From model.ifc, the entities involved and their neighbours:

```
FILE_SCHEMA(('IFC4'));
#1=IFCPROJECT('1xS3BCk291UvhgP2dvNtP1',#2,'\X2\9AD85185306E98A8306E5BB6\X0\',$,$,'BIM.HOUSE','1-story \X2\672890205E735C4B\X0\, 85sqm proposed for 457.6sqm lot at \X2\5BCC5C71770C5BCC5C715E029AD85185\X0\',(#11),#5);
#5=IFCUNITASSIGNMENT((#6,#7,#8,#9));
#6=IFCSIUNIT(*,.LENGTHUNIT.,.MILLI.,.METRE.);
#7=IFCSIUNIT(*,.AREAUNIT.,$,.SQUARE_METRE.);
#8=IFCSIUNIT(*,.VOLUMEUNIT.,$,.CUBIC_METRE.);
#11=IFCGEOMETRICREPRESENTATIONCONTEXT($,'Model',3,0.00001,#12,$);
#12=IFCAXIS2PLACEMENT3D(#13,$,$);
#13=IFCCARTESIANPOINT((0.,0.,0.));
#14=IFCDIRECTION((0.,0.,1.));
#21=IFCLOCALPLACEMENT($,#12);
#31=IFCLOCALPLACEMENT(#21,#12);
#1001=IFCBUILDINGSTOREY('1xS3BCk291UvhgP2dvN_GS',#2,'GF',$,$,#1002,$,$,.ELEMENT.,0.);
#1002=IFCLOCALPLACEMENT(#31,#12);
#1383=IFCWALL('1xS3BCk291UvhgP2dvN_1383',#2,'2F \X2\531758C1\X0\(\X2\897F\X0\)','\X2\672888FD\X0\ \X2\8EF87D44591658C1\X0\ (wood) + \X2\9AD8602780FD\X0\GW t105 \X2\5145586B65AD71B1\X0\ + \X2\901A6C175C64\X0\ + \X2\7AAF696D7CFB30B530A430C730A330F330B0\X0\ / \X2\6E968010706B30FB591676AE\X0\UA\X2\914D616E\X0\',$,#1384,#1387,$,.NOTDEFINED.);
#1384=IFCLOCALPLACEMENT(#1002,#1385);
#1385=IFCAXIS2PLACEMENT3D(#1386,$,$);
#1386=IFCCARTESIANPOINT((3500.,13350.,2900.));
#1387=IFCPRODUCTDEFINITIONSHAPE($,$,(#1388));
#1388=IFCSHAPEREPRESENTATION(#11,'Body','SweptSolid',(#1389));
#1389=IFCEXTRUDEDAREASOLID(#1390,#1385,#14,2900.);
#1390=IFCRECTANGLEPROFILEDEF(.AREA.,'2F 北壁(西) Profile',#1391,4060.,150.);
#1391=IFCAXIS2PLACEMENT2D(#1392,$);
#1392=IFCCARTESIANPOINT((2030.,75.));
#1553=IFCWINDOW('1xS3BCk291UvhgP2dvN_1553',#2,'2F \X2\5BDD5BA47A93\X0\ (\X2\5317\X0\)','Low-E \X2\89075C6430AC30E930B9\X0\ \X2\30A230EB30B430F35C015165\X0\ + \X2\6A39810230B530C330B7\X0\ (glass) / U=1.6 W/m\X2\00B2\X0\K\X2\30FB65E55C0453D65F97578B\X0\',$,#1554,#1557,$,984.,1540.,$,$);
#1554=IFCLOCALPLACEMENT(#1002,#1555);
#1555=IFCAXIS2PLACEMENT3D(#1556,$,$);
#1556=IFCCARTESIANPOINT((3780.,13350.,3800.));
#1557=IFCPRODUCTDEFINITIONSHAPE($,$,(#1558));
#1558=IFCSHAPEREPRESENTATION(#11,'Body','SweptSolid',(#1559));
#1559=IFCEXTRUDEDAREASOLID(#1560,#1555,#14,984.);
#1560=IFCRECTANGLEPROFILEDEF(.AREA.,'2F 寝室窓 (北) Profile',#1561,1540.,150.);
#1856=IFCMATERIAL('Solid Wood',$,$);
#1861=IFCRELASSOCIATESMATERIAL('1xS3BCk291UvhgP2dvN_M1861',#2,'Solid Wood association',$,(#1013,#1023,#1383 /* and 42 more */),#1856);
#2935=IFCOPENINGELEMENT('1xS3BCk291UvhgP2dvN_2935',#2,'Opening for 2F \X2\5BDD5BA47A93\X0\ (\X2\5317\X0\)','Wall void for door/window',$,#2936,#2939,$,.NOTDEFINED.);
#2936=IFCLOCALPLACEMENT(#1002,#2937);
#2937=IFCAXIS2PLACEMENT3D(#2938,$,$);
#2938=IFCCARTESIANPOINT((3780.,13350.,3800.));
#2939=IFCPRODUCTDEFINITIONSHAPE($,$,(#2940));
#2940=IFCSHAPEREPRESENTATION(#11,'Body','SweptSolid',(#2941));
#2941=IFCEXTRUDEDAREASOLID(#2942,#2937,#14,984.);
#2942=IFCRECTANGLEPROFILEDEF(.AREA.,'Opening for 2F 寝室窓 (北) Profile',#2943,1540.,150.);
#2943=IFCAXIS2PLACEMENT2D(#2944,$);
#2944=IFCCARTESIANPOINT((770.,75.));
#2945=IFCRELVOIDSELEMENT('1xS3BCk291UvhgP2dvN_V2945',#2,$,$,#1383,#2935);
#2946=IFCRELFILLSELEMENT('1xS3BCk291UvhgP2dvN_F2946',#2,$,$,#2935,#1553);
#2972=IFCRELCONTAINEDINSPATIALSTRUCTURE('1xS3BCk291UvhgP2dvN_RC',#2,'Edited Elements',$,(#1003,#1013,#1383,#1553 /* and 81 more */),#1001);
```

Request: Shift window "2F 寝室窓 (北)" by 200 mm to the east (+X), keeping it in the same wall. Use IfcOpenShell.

```python
import ifcopenshell
import ifcopenshell.api.geometry
import ifcopenshell.util.placement

model = ifcopenshell.open("model.ifc")

window = model.by_guid("1xS3BCk291UvhgP2dvN_1553")
opening = window.FillsVoids[0].RelatingOpeningElement
wall = opening.VoidsElements[0].RelatingBuildingElement

wall_matrix = ifcopenshell.util.placement.get_local_placement(wall.ObjectPlacement)
shift = wall_matrix[:3, 0] * 200.0
before = ifcopenshell.util.placement.get_local_placement(window.ObjectPlacement)[:3, 3].copy()

# The window is not placed relative to its opening, so move both.
for product in (opening, window):
    matrix = ifcopenshell.util.placement.get_local_placement(product.ObjectPlacement)
    matrix[:3, 3] += shift
    ifcopenshell.api.geometry.edit_object_placement(model, product=product, matrix=matrix, is_si=False)

after = ifcopenshell.util.placement.get_local_placement(window.ObjectPlacement)[:3, 3]
print("window moved by", (after - before).round(3) + 0.0)

model.write("model_edited.ifc")
```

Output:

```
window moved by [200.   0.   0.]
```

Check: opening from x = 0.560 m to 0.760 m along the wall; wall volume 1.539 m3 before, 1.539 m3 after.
